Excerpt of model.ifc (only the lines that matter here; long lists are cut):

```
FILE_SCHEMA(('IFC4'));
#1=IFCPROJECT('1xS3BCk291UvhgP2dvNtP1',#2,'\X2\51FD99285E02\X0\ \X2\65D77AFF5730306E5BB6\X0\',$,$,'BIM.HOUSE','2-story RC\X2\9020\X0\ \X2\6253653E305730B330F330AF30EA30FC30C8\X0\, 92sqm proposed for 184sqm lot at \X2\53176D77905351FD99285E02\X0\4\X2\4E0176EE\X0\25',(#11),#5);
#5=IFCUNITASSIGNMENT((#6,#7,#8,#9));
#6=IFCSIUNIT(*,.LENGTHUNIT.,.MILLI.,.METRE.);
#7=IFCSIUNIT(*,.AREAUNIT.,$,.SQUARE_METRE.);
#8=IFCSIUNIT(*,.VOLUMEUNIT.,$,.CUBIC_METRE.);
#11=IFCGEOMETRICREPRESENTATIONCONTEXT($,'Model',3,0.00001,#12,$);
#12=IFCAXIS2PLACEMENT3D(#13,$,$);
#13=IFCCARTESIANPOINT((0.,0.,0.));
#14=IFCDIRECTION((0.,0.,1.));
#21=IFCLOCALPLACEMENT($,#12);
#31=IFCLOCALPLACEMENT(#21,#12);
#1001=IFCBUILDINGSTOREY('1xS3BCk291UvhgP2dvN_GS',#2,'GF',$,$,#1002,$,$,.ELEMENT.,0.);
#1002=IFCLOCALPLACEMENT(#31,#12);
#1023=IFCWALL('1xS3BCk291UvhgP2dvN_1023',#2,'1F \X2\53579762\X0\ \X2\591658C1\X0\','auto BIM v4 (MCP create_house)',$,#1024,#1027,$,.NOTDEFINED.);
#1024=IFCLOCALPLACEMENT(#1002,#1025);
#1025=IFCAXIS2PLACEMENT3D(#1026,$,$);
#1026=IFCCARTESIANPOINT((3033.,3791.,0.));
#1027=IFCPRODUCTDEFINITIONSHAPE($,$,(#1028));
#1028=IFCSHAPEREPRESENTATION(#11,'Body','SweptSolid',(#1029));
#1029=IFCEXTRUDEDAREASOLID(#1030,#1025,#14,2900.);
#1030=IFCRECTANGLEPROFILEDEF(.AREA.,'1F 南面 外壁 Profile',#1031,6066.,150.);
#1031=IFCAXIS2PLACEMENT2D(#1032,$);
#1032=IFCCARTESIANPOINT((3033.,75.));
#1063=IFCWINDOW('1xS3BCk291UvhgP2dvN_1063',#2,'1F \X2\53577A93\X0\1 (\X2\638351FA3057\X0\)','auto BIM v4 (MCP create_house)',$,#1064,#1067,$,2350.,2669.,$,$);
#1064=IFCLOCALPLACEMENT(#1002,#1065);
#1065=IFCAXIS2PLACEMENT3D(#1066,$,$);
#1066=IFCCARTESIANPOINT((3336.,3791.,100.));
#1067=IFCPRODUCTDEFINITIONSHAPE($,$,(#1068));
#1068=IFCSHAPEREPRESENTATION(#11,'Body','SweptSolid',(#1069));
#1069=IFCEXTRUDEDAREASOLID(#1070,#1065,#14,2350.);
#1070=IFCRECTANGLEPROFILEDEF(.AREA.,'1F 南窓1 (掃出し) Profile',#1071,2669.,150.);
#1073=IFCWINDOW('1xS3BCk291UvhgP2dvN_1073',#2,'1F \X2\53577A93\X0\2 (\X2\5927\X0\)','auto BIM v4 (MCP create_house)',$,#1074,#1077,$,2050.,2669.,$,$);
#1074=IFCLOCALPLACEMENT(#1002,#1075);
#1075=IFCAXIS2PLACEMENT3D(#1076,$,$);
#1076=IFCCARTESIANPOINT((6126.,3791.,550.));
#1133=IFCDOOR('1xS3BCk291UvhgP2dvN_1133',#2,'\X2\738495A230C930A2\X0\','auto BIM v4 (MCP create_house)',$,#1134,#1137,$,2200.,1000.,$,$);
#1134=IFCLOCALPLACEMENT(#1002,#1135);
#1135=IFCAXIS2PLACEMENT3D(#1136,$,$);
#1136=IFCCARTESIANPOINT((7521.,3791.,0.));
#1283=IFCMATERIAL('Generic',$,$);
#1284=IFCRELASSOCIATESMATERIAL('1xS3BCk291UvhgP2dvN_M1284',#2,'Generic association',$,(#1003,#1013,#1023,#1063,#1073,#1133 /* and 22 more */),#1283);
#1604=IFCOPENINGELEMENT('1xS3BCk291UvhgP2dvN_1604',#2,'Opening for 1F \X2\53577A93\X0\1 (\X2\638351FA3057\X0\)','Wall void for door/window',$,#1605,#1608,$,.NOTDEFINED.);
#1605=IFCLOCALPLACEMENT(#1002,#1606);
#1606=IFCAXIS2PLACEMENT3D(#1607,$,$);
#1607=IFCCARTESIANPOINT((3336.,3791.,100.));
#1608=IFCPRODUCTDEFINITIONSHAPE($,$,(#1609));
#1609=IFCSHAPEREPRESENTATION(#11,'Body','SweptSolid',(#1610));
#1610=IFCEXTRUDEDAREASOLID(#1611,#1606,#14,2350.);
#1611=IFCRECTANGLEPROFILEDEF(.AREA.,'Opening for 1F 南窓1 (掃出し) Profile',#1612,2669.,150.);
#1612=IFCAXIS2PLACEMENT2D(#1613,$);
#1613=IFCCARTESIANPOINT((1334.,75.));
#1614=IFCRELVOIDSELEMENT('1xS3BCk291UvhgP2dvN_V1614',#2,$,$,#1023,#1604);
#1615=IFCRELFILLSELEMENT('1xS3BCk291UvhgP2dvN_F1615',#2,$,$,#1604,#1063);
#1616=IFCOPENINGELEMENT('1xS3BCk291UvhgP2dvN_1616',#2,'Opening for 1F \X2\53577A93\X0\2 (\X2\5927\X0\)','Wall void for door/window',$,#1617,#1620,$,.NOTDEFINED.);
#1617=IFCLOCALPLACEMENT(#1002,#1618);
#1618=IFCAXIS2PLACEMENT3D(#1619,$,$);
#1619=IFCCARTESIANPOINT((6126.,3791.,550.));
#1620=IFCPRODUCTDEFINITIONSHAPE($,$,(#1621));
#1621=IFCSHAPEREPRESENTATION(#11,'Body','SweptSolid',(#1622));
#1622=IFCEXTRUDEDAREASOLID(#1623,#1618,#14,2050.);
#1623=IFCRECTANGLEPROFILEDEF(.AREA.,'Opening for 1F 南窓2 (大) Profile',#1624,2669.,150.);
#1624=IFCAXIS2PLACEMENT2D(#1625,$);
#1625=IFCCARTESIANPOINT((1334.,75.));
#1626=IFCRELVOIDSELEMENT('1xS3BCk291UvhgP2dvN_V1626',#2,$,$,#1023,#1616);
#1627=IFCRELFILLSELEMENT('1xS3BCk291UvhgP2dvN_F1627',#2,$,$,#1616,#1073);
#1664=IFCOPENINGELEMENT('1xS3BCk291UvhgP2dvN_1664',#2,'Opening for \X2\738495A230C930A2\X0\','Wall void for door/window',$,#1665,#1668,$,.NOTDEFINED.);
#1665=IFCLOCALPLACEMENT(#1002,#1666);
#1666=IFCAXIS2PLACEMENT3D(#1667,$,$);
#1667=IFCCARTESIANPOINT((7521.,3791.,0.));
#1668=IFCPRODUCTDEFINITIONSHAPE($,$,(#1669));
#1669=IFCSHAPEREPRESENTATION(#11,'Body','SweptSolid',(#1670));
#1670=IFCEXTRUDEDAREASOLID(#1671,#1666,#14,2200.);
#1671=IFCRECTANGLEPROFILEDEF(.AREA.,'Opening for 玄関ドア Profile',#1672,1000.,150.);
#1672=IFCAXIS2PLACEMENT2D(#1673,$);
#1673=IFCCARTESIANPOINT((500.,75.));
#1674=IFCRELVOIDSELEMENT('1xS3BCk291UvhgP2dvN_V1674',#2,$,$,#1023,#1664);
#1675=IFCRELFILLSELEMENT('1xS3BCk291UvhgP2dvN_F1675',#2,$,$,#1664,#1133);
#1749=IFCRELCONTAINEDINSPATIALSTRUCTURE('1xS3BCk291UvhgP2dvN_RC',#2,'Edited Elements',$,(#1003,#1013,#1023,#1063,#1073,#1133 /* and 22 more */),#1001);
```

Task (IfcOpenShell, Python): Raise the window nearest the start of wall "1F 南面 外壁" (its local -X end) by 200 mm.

```python
import numpy as np
import ifcopenshell
import ifcopenshell.api.geometry
import ifcopenshell.util.placement
import ifcopenshell.util.unit

model = ifcopenshell.open("model.ifc")
unit_scale = ifcopenshell.util.unit.calculate_unit_scale(model)

window = model.by_id(1063)
opening = window.FillsVoids[0].RelatingOpeningElement
dz = 200.0

shift = np.array([0.0, 0.0, dz])
# The window is not placed relative to its opening, so move both.
for product in (opening, window):
    matrix = ifcopenshell.util.placement.get_local_placement(product.ObjectPlacement)
    matrix[:3, 3] += shift
    ifcopenshell.api.geometry.edit_object_placement(model, product=product, matrix=matrix, is_si=False)

print(f"moved by {dz * unit_scale:+.3f} m")

model.write("model_edited.ifc")
```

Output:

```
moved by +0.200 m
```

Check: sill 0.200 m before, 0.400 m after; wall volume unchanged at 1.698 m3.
